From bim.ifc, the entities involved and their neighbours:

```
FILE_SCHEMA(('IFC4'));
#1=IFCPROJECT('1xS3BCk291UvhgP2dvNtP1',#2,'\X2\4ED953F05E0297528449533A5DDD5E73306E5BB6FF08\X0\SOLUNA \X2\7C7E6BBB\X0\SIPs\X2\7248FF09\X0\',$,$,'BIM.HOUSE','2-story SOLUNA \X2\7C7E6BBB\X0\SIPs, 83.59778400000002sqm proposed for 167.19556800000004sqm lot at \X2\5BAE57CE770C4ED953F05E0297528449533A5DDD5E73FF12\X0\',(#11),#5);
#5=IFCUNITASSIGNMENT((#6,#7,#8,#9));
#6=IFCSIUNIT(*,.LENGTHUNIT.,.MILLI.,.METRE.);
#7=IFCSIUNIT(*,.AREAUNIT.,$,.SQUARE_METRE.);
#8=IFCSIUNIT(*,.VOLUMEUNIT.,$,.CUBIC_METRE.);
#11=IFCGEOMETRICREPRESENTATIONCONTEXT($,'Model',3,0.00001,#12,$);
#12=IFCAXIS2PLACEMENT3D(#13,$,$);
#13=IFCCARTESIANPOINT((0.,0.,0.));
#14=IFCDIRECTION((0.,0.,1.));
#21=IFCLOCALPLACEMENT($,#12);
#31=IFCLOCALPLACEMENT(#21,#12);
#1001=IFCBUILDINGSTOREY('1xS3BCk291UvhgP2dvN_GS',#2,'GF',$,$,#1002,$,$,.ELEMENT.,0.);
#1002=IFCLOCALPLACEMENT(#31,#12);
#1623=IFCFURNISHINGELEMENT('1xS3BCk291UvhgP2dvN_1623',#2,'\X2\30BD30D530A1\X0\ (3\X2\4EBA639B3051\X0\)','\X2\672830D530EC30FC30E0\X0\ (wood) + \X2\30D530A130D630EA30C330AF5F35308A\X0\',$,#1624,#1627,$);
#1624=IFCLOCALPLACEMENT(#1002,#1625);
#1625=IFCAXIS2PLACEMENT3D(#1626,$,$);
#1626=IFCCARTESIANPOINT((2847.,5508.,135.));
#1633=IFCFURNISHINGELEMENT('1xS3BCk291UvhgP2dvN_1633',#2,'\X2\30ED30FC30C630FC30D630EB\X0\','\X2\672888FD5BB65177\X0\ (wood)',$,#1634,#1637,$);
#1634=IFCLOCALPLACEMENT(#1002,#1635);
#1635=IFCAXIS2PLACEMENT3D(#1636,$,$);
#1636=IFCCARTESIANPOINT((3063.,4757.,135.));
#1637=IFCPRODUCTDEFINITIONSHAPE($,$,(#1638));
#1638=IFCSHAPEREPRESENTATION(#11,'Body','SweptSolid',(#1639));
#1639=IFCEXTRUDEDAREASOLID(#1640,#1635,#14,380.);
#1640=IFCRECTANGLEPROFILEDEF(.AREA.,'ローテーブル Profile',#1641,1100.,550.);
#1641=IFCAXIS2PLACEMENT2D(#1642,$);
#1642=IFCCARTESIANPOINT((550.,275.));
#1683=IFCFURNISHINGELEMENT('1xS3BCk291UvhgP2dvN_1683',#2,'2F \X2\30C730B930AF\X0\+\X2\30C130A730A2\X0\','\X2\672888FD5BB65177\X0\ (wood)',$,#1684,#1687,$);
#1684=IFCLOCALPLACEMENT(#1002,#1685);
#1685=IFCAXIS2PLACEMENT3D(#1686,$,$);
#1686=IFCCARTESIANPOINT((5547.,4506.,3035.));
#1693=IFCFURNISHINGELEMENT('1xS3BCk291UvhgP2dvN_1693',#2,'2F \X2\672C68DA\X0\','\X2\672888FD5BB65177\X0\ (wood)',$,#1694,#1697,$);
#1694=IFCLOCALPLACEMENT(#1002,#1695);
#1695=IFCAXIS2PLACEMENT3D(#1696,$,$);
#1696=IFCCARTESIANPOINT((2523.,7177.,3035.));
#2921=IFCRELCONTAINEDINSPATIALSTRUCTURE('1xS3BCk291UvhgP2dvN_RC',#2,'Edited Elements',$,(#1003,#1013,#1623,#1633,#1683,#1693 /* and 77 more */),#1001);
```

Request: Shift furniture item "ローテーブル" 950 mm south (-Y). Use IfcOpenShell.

```python
import ifcopenshell
import ifcopenshell.api.geometry
import ifcopenshell.util.placement
import ifcopenshell.util.unit

model = ifcopenshell.open("bim.ifc")
unit_scale = ifcopenshell.util.unit.calculate_unit_scale(model)

item = model.by_guid("1xS3BCk291UvhgP2dvN_1633")
matrix = ifcopenshell.util.placement.get_local_placement(item.ObjectPlacement)
matrix[1, 3] -= 0.95 / unit_scale
ifcopenshell.api.geometry.edit_object_placement(model, product=item, matrix=matrix, is_si=False)

print(ifcopenshell.util.placement.get_local_placement(item.ObjectPlacement).round(3) + 0.0)

model.write("bim-out.ifc")
```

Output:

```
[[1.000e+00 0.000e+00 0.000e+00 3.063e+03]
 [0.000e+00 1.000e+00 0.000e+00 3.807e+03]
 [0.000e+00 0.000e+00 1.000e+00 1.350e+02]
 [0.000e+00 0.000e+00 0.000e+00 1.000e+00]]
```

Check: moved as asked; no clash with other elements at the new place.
